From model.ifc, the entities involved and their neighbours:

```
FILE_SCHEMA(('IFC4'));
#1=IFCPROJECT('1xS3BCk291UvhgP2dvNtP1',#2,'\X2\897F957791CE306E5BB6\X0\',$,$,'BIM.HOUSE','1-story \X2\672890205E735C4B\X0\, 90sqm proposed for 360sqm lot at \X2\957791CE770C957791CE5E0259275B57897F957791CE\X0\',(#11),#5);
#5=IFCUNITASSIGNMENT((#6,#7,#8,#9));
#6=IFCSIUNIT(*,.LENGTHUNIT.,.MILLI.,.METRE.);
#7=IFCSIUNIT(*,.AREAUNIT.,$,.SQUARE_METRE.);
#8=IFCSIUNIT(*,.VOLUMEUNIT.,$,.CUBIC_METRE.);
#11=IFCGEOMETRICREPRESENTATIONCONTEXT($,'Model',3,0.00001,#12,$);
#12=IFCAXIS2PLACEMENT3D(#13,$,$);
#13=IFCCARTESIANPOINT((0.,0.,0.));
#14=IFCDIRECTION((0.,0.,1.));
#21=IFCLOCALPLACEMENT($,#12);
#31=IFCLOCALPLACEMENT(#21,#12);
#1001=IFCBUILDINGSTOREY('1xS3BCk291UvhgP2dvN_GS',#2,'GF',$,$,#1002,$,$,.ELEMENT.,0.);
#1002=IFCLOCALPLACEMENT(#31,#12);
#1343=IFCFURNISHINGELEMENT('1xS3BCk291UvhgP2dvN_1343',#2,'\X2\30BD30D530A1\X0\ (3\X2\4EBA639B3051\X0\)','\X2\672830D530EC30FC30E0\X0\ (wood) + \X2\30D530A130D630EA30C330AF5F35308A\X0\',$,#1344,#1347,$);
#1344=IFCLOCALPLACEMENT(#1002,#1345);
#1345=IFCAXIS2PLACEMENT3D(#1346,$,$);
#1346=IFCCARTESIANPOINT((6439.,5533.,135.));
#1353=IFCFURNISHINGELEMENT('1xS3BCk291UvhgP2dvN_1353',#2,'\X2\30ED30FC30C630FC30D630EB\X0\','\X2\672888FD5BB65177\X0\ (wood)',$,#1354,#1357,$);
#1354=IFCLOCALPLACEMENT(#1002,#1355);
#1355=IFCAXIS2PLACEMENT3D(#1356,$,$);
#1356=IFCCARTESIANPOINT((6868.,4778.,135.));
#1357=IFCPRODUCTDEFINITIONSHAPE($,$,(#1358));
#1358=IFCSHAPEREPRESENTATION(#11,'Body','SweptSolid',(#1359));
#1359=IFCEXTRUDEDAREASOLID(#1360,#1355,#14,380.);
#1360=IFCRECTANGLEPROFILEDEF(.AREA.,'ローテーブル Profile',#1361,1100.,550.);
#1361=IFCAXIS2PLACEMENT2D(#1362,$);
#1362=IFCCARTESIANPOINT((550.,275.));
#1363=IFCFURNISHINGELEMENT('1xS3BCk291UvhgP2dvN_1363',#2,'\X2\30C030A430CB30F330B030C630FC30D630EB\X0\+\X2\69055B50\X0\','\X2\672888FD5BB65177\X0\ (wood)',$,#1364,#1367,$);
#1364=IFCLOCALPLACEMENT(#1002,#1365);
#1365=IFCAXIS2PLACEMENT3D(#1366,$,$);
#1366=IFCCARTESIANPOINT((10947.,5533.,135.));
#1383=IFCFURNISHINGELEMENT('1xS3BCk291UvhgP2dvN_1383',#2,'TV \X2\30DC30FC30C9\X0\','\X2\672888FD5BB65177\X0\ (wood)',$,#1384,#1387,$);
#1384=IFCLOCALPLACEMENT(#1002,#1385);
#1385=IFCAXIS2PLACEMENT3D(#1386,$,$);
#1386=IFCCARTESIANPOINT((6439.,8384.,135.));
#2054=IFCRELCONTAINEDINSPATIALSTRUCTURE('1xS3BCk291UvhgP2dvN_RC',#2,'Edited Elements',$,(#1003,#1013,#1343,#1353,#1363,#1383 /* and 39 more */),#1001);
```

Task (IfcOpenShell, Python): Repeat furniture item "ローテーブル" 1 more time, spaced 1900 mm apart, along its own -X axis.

```python
import ifcopenshell
import ifcopenshell.api.geometry
import ifcopenshell.api.root
import ifcopenshell.util.element
import ifcopenshell.util.placement

model = ifcopenshell.open("model.ifc")


def reuse_history(source, copy):
    """copy_class also copies each property set's owner history, people and application; keep the originals."""
    for rel in copy.IsDefinedBy:
        if rel.is_a("IfcRelDefinesByProperties") and (history := rel.RelatingPropertyDefinition.OwnerHistory):
            rel.RelatingPropertyDefinition.OwnerHistory = source.OwnerHistory
            ifcopenshell.util.element.remove_deep2(model, history)


source = model.by_id(1353)
base = ifcopenshell.util.placement.get_local_placement(source.ObjectPlacement)
step = -base[:3, 0] * 1900.0

for i in range(1, 2):
    copy = ifcopenshell.api.root.copy_class(model, product=source)
    copy.Representation = ifcopenshell.util.element.copy_deep(
        model, source.Representation, exclude=["IfcGeometricRepresentationContext", "IfcRepresentationMap"]
    )
    reuse_history(source, copy)
    matrix = base.copy()
    matrix[:3, 3] += i * step
    print("added at", matrix[:3, 3].round(3) + 0.0)
    ifcopenshell.api.geometry.edit_object_placement(model, product=copy, matrix=matrix, is_si=False)

model.write("model_rev.ifc")
```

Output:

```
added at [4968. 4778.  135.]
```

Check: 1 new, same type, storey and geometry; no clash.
